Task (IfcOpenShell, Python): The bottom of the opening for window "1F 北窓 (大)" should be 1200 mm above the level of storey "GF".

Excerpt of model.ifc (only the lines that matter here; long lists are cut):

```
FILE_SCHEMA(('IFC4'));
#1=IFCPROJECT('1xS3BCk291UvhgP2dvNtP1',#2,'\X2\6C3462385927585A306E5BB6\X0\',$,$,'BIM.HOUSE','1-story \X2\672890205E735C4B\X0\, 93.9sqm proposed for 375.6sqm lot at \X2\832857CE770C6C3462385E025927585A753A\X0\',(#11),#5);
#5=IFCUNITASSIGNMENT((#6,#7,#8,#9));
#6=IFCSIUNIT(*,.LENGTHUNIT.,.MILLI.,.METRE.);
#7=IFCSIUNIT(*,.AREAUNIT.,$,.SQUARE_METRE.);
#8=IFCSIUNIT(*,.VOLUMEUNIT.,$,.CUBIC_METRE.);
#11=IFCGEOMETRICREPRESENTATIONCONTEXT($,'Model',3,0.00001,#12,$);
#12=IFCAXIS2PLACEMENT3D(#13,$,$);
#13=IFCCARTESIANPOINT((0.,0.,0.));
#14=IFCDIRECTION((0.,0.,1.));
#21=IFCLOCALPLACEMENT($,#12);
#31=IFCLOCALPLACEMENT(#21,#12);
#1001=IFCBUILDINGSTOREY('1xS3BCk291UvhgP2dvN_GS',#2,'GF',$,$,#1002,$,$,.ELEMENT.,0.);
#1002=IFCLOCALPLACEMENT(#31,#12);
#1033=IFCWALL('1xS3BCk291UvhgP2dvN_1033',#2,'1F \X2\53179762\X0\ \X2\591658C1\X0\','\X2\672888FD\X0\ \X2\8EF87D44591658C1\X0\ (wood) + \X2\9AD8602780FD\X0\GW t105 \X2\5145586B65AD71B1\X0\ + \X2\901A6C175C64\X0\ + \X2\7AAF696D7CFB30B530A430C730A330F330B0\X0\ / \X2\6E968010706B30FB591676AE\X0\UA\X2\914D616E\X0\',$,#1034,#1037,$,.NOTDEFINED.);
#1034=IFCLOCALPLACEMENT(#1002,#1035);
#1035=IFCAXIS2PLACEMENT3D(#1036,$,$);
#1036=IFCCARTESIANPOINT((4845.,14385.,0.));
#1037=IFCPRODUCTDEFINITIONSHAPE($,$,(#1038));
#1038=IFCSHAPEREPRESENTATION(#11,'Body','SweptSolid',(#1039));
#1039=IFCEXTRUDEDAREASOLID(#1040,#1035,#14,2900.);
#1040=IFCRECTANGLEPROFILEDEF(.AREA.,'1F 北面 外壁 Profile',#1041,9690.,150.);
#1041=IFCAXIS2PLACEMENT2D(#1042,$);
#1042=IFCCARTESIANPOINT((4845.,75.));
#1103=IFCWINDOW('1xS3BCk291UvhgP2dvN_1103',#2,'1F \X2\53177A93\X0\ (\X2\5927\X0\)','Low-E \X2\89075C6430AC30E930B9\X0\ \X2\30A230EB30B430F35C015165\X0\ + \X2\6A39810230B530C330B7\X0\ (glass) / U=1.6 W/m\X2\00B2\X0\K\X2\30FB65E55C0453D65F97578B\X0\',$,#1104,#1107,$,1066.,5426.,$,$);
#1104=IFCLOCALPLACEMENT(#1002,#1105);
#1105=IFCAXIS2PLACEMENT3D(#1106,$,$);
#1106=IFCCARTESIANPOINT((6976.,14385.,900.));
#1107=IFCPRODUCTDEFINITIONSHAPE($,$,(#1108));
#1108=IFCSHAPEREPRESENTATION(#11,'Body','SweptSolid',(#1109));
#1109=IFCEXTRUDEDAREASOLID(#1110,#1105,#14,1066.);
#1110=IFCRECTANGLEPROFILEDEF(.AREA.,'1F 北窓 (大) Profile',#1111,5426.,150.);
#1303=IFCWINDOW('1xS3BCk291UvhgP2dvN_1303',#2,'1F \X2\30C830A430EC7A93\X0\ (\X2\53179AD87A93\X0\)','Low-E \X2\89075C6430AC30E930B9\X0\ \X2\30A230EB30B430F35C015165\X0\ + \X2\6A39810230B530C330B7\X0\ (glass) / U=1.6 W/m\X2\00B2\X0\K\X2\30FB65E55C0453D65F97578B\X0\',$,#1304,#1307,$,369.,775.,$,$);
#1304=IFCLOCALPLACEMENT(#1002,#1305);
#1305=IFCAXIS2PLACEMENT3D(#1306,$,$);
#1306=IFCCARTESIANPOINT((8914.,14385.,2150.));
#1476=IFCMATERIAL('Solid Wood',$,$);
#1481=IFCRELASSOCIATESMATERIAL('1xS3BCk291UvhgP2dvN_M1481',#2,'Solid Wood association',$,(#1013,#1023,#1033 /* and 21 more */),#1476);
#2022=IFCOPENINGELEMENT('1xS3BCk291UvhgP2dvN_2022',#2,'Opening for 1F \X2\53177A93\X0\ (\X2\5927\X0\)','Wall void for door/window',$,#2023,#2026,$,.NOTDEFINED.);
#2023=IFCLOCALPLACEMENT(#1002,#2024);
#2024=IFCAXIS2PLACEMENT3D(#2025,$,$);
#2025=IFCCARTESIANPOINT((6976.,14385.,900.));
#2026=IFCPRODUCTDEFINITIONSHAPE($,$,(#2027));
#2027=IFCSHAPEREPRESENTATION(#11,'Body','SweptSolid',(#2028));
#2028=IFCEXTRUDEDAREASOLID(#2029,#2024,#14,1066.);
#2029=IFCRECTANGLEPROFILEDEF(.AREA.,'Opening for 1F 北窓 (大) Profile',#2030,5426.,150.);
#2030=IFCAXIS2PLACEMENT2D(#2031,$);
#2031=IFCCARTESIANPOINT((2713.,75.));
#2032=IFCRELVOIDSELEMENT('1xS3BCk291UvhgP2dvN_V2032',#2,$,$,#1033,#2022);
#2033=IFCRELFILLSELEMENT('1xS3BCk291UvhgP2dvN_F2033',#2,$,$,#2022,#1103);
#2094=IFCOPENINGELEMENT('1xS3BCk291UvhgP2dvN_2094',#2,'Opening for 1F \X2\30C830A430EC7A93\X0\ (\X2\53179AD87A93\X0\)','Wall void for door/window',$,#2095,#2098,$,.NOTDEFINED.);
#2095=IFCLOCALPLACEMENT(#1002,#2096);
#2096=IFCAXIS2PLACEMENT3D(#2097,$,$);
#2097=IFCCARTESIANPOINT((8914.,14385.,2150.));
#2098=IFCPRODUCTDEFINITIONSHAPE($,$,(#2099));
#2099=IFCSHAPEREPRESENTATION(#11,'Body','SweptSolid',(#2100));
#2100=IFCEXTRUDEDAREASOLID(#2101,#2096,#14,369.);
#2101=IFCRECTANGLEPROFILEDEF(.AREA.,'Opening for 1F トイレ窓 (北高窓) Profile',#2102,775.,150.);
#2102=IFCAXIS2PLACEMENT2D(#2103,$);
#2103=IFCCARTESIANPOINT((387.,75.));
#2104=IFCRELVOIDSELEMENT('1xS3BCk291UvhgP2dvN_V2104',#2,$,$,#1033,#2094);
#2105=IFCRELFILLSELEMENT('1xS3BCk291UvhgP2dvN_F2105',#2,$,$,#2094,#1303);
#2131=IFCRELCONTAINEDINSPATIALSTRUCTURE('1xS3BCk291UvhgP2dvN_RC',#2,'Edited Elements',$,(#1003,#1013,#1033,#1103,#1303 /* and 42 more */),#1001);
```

```python
import numpy as np
import ifcopenshell
import ifcopenshell.api.geometry
import ifcopenshell.geom
import ifcopenshell.util.element
import ifcopenshell.util.placement
import ifcopenshell.util.shape
import ifcopenshell.util.unit

model = ifcopenshell.open("model.ifc")
unit_scale = ifcopenshell.util.unit.calculate_unit_scale(model)

window = model.by_guid("1xS3BCk291UvhgP2dvN_1103")
opening = window.FillsVoids[0].RelatingOpeningElement
storey = ifcopenshell.util.element.get_container(window, ifc_class="IfcBuildingStorey")
level = ifcopenshell.util.placement.get_local_placement(storey.ObjectPlacement)[2, 3]

# The opening's origin need not be at the sill, so measure its lowest point.
shape = ifcopenshell.geom.create_shape(ifcopenshell.geom.settings(), opening)
bottom = ifcopenshell.util.shape.get_shape_bottom_elevation(shape, shape.geometry) / unit_scale
dz = level + 1.2 / unit_scale - bottom

shift = np.array([0.0, 0.0, dz])
# The window is not placed relative to its opening, so move both.
for product in (opening, window):
    matrix = ifcopenshell.util.placement.get_local_placement(product.ObjectPlacement)
    matrix[:3, 3] += shift
    ifcopenshell.api.geometry.edit_object_placement(model, product=product, matrix=matrix, is_si=False)

print(f"moved by {dz * unit_scale:+.3f} m")

model.write("model_updated.ifc")
```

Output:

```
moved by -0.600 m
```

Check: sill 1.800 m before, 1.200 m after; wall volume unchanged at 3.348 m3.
